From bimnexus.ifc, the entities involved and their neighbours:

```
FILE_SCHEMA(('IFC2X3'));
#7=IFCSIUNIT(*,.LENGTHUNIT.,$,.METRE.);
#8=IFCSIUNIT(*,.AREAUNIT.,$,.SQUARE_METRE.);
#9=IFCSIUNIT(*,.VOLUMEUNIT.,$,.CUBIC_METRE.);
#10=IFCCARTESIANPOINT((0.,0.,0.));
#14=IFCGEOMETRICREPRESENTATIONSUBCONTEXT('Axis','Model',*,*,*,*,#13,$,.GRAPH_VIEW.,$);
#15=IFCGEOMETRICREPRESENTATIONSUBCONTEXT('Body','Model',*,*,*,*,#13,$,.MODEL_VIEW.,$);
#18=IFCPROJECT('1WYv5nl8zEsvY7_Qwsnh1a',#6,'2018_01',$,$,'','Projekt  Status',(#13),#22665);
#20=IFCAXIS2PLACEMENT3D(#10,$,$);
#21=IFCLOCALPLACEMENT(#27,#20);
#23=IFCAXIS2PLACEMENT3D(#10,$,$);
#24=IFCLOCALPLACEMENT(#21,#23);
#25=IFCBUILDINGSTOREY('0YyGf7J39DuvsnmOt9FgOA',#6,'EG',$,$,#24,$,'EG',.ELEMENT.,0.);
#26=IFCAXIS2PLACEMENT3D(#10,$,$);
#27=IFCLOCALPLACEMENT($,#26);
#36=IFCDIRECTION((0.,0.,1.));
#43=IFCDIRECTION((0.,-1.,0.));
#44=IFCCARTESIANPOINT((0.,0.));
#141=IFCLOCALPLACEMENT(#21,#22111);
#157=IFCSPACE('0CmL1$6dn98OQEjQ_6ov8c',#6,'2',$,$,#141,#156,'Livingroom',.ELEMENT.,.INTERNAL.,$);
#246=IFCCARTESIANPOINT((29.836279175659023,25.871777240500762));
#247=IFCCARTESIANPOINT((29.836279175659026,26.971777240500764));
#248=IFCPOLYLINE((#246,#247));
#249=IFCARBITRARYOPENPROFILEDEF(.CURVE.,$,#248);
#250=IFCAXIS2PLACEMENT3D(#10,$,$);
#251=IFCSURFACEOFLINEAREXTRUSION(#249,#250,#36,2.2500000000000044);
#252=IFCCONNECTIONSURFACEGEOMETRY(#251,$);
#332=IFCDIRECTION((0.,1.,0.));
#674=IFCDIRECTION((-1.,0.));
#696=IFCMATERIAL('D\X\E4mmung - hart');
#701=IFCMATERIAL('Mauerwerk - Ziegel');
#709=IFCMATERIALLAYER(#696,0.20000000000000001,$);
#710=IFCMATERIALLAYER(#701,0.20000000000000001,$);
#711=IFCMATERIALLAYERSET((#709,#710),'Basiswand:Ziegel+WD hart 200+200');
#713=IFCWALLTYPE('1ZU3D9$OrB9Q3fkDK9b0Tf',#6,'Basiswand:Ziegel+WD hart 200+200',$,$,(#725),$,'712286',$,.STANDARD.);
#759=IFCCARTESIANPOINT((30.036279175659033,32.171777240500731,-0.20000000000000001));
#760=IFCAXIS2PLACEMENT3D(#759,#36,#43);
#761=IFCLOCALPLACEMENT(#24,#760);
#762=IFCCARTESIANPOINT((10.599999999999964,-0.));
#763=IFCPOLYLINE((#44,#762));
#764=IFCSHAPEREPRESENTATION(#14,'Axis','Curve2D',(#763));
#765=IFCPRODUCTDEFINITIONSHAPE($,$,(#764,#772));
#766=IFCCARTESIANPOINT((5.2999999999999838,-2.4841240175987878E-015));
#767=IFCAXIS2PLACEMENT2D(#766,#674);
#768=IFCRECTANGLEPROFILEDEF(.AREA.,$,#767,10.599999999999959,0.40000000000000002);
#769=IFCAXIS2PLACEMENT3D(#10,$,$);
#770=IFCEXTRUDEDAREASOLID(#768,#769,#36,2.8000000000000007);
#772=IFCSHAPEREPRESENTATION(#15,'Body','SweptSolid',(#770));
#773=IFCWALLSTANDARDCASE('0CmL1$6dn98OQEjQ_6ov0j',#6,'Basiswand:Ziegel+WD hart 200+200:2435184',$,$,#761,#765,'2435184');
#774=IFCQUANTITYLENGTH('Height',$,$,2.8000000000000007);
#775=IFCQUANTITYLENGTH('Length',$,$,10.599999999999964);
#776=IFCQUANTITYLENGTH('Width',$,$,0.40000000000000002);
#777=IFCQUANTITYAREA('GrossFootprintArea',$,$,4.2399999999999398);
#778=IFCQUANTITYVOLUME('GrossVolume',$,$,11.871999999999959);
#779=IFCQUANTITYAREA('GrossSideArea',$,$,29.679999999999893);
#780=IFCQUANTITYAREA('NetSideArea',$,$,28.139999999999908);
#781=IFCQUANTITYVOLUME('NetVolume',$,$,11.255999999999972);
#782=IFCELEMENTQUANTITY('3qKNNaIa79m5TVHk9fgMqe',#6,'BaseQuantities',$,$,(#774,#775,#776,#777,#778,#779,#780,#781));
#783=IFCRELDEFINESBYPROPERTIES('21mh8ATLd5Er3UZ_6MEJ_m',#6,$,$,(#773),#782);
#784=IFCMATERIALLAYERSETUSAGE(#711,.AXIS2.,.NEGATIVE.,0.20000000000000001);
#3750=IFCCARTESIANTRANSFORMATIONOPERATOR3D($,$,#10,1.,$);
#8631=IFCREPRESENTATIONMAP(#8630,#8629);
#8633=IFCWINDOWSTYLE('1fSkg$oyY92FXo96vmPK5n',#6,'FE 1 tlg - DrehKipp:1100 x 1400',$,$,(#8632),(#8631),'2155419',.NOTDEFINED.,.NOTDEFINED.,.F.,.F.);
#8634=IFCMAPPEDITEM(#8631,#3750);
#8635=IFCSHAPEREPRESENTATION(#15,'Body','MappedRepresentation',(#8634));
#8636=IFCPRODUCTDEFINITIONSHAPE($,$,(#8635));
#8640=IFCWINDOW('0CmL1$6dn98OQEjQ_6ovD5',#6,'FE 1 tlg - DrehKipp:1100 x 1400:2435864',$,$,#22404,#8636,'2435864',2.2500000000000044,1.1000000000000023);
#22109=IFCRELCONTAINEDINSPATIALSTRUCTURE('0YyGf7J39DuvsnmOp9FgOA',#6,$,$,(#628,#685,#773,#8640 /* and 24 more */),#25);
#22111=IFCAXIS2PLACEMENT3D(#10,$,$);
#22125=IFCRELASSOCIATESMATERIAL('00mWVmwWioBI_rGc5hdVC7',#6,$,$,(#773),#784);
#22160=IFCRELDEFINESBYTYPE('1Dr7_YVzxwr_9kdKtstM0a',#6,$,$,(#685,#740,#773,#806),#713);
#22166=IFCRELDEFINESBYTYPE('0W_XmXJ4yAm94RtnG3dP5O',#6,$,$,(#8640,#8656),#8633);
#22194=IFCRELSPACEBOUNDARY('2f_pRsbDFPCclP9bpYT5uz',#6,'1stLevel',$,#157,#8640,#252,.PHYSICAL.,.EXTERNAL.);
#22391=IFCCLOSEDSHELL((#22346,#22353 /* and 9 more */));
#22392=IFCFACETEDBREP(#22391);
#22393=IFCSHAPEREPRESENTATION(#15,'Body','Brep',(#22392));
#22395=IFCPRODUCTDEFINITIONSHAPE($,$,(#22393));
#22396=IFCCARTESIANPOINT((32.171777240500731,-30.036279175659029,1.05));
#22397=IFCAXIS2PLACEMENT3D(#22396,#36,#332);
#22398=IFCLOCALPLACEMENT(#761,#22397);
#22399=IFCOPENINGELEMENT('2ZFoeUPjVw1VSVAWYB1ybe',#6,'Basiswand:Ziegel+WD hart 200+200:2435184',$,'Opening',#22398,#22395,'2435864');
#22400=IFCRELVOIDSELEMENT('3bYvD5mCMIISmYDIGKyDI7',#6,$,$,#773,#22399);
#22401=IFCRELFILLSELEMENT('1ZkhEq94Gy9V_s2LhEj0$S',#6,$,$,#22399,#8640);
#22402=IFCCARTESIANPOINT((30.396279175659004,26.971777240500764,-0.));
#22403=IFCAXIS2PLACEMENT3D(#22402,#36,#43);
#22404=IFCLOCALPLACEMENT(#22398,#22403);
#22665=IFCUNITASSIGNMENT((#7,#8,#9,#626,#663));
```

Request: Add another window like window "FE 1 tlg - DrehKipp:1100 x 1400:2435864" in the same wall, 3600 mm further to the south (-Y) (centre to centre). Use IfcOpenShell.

```python
import numpy as np
import ifcopenshell
import ifcopenshell.api.feature
import ifcopenshell.api.geometry
import ifcopenshell.api.pset
import ifcopenshell.api.root
import ifcopenshell.geom
import ifcopenshell.util.element
import ifcopenshell.util.placement
import ifcopenshell.util.shape
import ifcopenshell.util.unit

model = ifcopenshell.open("bimnexus.ifc")
unit_scale = ifcopenshell.util.unit.calculate_unit_scale(model)
area_scale = ifcopenshell.util.unit.calculate_unit_scale(model, "AREAUNIT")
volume_scale = ifcopenshell.util.unit.calculate_unit_scale(model, "VOLUMEUNIT")
settings = ifcopenshell.geom.settings()


def volume(element):
    """Net volume in cubic metres, openings subtracted."""
    shape = ifcopenshell.geom.create_shape(settings, element)
    return ifcopenshell.util.shape.get_volume(shape.geometry)


def reuse_history(source, copy):
    """copy_class also copies each property set's owner history, people and application; keep the originals."""
    for rel in copy.IsDefinedBy:
        if rel.is_a("IfcRelDefinesByProperties") and (history := rel.RelatingPropertyDefinition.OwnerHistory):
            rel.RelatingPropertyDefinition.OwnerHistory = source.OwnerHistory
            ifcopenshell.util.element.remove_deep2(model, history)


window = model.by_guid("0CmL1$6dn98OQEjQ_6ovD5")
opening = window.FillsVoids[0].RelatingOpeningElement
wall = opening.VoidsElements[0].RelatingBuildingElement
before = volume(wall)
shift = ifcopenshell.util.placement.get_local_placement(wall.ObjectPlacement)[:3, 0] * 3.6 / unit_scale

# copy_class copies the void relationship, type, container and properties, but no geometry.
new_opening = ifcopenshell.api.root.copy_class(model, product=opening)
new_opening.Representation = ifcopenshell.util.element.copy_deep(
    model, opening.Representation, exclude=["IfcGeometricRepresentationContext", "IfcRepresentationMap"]
)
new_opening.Name = "Basiswand:Ziegel+WD hart 200+200"
new_opening.Tag = None
new_window = ifcopenshell.api.root.copy_class(model, product=window)
new_window.Representation = ifcopenshell.util.element.copy_deep(
    model, window.Representation, exclude=["IfcGeometricRepresentationContext", "IfcRepresentationMap"]
)
new_window.Name = "FE 1 tlg - DrehKipp:1100 x 1400"
new_window.Tag = None
reuse_history(window, new_window)
fills = ifcopenshell.api.feature.add_filling(model, opening=new_opening, element=new_window)
fills.OwnerHistory = new_window.OwnerHistory  # required in IFC2X3

for old, new in ((opening, new_opening), (window, new_window)):
    matrix = ifcopenshell.util.placement.get_local_placement(old.ObjectPlacement)
    matrix[:3, 3] += shift
    ifcopenshell.api.geometry.edit_object_placement(model, product=new, matrix=matrix, is_si=False)

# The copied space boundaries still share their surfaces with the original.
for rel in new_window.ProvidesBoundaries:
    if rel.ConnectionGeometry:
        rel.ConnectionGeometry = ifcopenshell.util.element.copy_deep(model, rel.ConnectionGeometry)

# Space boundary surfaces are stored in each space's coordinates; move them too.
for rel in new_window.ProvidesBoundaries:
    if not rel.ConnectionGeometry:
        continue
    surface = rel.ConnectionGeometry.SurfaceOnRelatingElement
    space_matrix = ifcopenshell.util.placement.get_local_placement(rel.RelatingSpace.ObjectPlacement)
    point = np.array(surface.Position.Location.Coordinates) + space_matrix[:3, :3].T @ shift
    surface.Position = model.createIfcAxis2Placement3D(
        model.createIfcCartesianPoint(point.tolist()), surface.Position.Axis, surface.Position.RefDirection
    )

after = volume(wall)
thickness = 0.4  # wall thickness in metres

# Update the wall's stored quantities.
qto = model.by_id(ifcopenshell.util.element.get_pset(wall, "BaseQuantities", should_inherit=False)["id"])
ifcopenshell.api.pset.edit_qto(model, qto=qto, properties={
    "NetSideArea": after / thickness / area_scale,
    "NetVolume": after / volume_scale,
})

print(f"wall volume {before:.3f} -> {after:.3f} m3")

model.write("bimnexus-out.ifc")
```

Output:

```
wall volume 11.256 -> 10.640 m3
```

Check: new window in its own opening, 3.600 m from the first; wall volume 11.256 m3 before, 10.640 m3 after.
